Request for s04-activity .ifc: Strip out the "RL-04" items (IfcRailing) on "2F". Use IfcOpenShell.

First a look at what the model holds.

```python
import ifcopenshell
import ifcopenshell.util.element

model = ifcopenshell.open("s04-activity .ifc")
print(model.schema)
storey = next(s for s in model.by_type("IfcBuildingStorey") if s.Name == "2F")
railings = [e for e in ifcopenshell.util.element.get_decomposition(storey) if e.is_a("IfcRailing")]
seen = {}
for e in railings:
    element_type = ifcopenshell.util.element.get_type(e)
    name = element_type.Name if element_type not in (None, e) else None
    seen[name] = seen.get(name, 0) + 1
for name, count in sorted(seen.items(), key=str):
    print(count, "x", name)
```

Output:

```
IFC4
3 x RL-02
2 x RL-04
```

```python
import ifcopenshell
import ifcopenshell.api.root
import ifcopenshell.util.element

model = ifcopenshell.open("s04-activity .ifc")

storey = next(s for s in model.by_type("IfcBuildingStorey") if s.Name == "2F")
railings = [e for e in ifcopenshell.util.element.get_decomposition(storey) if e.is_a("IfcRailing")]
targets = [e for e in railings if (t := ifcopenshell.util.element.get_type(e)) not in (None, e) and t.Name == "RL-04"]

for e in targets:
    ifcopenshell.api.root.remove_product(model, product=e)
print(len(targets), "removed")

model.write("s04-activity _updated.ifc")
```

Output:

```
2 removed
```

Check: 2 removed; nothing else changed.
